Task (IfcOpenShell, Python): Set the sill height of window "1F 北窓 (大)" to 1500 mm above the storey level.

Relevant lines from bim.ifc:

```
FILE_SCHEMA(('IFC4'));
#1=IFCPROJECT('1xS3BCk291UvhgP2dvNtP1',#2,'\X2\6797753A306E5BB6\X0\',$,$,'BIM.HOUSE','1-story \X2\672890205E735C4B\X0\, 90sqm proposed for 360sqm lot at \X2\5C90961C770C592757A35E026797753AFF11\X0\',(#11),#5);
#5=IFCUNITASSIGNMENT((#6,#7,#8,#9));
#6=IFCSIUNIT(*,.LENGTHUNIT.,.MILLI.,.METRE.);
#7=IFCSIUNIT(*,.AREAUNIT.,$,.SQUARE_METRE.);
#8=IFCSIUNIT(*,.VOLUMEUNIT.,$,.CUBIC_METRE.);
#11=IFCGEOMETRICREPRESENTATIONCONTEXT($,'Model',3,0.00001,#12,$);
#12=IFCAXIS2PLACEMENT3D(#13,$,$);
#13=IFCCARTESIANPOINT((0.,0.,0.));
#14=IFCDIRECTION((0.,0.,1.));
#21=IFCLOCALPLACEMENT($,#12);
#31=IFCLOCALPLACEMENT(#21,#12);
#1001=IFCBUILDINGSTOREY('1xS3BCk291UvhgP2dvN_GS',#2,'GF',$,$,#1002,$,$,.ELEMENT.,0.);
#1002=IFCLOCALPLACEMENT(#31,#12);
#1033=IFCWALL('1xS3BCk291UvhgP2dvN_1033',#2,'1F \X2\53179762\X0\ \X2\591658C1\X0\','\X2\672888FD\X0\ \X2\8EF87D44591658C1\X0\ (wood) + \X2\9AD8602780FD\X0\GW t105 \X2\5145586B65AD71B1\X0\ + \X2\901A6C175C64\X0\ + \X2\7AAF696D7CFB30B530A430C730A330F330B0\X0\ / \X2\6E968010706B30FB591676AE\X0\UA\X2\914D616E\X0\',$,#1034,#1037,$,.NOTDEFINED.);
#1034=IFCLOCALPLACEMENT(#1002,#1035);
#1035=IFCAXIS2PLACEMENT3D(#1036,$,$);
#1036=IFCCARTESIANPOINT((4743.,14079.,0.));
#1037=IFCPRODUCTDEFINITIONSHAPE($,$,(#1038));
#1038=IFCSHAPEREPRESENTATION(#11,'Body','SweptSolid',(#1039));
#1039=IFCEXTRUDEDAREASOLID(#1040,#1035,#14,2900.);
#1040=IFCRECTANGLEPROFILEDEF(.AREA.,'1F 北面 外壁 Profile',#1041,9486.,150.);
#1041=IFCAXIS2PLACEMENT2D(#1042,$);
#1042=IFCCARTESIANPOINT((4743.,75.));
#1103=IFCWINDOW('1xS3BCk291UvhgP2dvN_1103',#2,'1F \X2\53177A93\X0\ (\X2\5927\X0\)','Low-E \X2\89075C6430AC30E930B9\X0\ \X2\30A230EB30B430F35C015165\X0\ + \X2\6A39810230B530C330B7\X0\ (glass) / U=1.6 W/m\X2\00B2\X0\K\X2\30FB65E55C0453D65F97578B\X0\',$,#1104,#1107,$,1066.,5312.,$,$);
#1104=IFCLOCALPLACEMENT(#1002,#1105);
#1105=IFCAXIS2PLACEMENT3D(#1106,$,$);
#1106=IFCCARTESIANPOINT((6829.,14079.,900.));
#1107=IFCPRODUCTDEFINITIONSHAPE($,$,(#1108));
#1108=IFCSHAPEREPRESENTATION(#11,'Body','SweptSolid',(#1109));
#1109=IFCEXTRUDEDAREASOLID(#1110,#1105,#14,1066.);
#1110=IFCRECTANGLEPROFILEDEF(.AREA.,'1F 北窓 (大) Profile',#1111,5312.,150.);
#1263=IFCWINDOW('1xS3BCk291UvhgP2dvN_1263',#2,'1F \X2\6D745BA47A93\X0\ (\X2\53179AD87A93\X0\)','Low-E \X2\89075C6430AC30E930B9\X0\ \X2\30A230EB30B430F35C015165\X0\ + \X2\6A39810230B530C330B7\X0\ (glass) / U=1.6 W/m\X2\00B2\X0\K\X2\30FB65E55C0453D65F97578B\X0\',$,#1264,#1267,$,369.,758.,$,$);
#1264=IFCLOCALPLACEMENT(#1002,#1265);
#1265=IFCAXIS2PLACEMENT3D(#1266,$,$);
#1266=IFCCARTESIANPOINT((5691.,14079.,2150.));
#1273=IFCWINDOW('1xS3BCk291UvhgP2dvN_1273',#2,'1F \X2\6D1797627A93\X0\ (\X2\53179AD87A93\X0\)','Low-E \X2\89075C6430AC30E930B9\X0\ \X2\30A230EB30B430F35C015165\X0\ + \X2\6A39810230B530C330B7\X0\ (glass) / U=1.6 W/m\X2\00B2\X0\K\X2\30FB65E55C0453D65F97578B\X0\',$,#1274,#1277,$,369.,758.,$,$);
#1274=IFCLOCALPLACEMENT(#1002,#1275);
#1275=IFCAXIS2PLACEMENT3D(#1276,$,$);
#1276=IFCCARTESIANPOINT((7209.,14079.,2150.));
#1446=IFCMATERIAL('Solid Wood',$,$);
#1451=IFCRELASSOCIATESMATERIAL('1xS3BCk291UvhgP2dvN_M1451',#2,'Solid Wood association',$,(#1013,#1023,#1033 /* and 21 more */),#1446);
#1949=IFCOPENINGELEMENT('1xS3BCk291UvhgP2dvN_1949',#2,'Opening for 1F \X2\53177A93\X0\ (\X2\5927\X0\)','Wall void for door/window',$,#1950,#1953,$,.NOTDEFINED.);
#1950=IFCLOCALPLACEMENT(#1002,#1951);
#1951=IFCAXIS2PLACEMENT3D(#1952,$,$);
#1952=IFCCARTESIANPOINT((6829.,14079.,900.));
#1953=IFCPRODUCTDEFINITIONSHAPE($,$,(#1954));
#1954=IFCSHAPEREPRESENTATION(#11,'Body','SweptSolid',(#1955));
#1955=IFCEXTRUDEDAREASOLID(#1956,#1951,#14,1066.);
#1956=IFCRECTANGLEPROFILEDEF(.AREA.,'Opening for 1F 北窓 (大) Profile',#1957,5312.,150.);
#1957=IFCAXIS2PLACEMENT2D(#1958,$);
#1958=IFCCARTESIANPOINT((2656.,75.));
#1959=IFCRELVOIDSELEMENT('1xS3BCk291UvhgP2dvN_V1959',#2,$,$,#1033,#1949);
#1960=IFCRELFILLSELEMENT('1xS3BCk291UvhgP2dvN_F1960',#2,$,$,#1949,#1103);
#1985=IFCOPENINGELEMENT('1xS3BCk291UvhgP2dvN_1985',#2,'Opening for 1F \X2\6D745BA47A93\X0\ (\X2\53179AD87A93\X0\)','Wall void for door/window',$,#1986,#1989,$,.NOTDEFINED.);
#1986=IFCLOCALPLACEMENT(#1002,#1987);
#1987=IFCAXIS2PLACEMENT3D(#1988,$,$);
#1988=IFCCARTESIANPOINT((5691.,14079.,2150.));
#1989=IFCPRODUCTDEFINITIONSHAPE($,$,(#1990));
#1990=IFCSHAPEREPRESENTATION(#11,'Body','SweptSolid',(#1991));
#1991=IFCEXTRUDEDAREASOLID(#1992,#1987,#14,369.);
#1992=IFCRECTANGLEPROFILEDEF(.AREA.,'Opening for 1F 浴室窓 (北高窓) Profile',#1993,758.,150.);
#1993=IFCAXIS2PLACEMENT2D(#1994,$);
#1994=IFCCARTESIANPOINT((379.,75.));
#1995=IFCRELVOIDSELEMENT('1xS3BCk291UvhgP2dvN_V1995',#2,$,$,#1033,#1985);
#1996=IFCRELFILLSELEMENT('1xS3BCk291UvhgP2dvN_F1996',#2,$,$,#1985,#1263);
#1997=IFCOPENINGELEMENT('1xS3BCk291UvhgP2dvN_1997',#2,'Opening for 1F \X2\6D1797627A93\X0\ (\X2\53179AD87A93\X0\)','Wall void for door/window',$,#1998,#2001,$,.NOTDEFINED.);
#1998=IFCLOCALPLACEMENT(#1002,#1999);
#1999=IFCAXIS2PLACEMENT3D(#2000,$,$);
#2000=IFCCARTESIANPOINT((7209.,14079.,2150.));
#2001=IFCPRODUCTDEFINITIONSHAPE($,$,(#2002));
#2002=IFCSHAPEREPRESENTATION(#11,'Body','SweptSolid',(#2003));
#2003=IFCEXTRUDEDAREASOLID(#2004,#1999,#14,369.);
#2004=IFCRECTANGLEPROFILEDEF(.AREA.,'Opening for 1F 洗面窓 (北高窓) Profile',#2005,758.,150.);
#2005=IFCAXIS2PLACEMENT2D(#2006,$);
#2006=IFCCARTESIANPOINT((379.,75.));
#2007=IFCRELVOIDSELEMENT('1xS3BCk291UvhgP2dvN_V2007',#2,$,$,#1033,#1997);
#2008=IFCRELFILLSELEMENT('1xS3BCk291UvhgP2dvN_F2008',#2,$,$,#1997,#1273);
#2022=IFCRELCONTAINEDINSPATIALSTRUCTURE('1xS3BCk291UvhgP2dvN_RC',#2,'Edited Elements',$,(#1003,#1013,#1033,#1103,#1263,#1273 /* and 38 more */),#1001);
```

```python
import numpy as np
import ifcopenshell
import ifcopenshell.api.geometry
import ifcopenshell.geom
import ifcopenshell.util.element
import ifcopenshell.util.placement
import ifcopenshell.util.shape
import ifcopenshell.util.unit

model = ifcopenshell.open("bim.ifc")
unit_scale = ifcopenshell.util.unit.calculate_unit_scale(model)

window = model.by_guid("1xS3BCk291UvhgP2dvN_1103")
opening = window.FillsVoids[0].RelatingOpeningElement
storey = ifcopenshell.util.element.get_container(window, ifc_class="IfcBuildingStorey")
level = ifcopenshell.util.placement.get_local_placement(storey.ObjectPlacement)[2, 3]

# The opening's origin need not be at the sill, so measure its lowest point.
shape = ifcopenshell.geom.create_shape(ifcopenshell.geom.settings(), opening)
bottom = ifcopenshell.util.shape.get_shape_bottom_elevation(shape, shape.geometry) / unit_scale
dz = level + 1.5 / unit_scale - bottom

shift = np.array([0.0, 0.0, dz])
# The window is not placed relative to its opening, so move both.
for product in (opening, window):
    matrix = ifcopenshell.util.placement.get_local_placement(product.ObjectPlacement)
    matrix[:3, 3] += shift
    ifcopenshell.api.geometry.edit_object_placement(model, product=product, matrix=matrix, is_si=False)

print(f"moved by {dz * unit_scale:+.3f} m")

model.write("bim_rev.ifc")
```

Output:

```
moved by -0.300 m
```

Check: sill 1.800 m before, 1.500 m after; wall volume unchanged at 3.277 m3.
